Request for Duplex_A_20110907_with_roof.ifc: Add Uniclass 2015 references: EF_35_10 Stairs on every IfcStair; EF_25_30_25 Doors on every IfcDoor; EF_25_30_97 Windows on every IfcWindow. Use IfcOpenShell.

First a look at what the model holds.

```python
import ifcopenshell

model = ifcopenshell.open("Duplex_A_20110907_with_roof.ifc")
print(model.schema)
print("classifications:", [c.Name for c in model.by_type("IfcClassification")])
for ifc_class in ("IfcDoor", "IfcRoof", "IfcStair", "IfcWall", "IfcWindow"):
    print(ifc_class, len(model.by_type(ifc_class)))
```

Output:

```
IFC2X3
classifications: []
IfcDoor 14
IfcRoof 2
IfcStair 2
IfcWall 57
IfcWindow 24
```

```python
import ifcopenshell
import ifcopenshell.api.classification

model = ifcopenshell.open("Duplex_A_20110907_with_roof.ifc")

# IFC2X3 requires Source and Edition and has no link from the project to the system.
system = model.create_entity("IfcClassification", Source="NBS", Edition="2015", Name="Uniclass 2015")

codes = {
    "IfcStair": ("EF_35_10", "Stairs"),
    "IfcDoor": ("EF_25_30_25", "Doors"),
    "IfcWindow": ("EF_25_30_97", "Windows"),
}
for ifc_class, (code, name) in codes.items():
    products = model.by_type(ifc_class)
    ifcopenshell.api.classification.add_reference(
        model, products=products, classification=system, identification=code, name=name
    )
    print(code, len(products))

model.write("Duplex_A_20110907_with_roof_edited.ifc")
```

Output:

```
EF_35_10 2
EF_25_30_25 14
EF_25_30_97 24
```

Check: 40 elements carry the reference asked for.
